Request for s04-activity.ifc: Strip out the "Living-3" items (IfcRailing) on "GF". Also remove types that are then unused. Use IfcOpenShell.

First a look at what the model holds.

```python
import ifcopenshell
import ifcopenshell.util.element

model = ifcopenshell.open("s04-activity.ifc")
print(model.schema)
storey = next(s for s in model.by_type("IfcBuildingStorey") if s.Name == "GF")
railings = [e for e in ifcopenshell.util.element.get_decomposition(storey) if e.is_a("IfcRailing")]
seen = {}
for e in railings:
    element_type = ifcopenshell.util.element.get_type(e)
    name = element_type.Name if element_type not in (None, e) else None
    seen[name] = seen.get(name, 0) + 1
for name, count in sorted(seen.items(), key=str):
    print(count, "x", name)
```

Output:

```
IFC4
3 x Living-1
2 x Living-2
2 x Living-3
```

```python
import ifcopenshell
import ifcopenshell.api.root
import ifcopenshell.util.element

model = ifcopenshell.open("s04-activity.ifc")

storey = next(s for s in model.by_type("IfcBuildingStorey") if s.Name == "GF")
railings = [e for e in ifcopenshell.util.element.get_decomposition(storey) if e.is_a("IfcRailing")]
targets = [e for e in railings if (t := ifcopenshell.util.element.get_type(e)) not in (None, e) and t.Name == "Living-3"]
types = {ifcopenshell.util.element.get_type(e) for e in targets} - {None, *targets}

for e in targets:
    ifcopenshell.api.root.remove_product(model, product=e)
print(len(targets), "removed")

unused = [t for t in types if not ifcopenshell.util.element.get_types(t)]
for t in unused:
    ifcopenshell.api.root.remove_product(model, product=t)
print(len(unused), "unused types removed")

model.write("s04-activity_edited.ifc")
```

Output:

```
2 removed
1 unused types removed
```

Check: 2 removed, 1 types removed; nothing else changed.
